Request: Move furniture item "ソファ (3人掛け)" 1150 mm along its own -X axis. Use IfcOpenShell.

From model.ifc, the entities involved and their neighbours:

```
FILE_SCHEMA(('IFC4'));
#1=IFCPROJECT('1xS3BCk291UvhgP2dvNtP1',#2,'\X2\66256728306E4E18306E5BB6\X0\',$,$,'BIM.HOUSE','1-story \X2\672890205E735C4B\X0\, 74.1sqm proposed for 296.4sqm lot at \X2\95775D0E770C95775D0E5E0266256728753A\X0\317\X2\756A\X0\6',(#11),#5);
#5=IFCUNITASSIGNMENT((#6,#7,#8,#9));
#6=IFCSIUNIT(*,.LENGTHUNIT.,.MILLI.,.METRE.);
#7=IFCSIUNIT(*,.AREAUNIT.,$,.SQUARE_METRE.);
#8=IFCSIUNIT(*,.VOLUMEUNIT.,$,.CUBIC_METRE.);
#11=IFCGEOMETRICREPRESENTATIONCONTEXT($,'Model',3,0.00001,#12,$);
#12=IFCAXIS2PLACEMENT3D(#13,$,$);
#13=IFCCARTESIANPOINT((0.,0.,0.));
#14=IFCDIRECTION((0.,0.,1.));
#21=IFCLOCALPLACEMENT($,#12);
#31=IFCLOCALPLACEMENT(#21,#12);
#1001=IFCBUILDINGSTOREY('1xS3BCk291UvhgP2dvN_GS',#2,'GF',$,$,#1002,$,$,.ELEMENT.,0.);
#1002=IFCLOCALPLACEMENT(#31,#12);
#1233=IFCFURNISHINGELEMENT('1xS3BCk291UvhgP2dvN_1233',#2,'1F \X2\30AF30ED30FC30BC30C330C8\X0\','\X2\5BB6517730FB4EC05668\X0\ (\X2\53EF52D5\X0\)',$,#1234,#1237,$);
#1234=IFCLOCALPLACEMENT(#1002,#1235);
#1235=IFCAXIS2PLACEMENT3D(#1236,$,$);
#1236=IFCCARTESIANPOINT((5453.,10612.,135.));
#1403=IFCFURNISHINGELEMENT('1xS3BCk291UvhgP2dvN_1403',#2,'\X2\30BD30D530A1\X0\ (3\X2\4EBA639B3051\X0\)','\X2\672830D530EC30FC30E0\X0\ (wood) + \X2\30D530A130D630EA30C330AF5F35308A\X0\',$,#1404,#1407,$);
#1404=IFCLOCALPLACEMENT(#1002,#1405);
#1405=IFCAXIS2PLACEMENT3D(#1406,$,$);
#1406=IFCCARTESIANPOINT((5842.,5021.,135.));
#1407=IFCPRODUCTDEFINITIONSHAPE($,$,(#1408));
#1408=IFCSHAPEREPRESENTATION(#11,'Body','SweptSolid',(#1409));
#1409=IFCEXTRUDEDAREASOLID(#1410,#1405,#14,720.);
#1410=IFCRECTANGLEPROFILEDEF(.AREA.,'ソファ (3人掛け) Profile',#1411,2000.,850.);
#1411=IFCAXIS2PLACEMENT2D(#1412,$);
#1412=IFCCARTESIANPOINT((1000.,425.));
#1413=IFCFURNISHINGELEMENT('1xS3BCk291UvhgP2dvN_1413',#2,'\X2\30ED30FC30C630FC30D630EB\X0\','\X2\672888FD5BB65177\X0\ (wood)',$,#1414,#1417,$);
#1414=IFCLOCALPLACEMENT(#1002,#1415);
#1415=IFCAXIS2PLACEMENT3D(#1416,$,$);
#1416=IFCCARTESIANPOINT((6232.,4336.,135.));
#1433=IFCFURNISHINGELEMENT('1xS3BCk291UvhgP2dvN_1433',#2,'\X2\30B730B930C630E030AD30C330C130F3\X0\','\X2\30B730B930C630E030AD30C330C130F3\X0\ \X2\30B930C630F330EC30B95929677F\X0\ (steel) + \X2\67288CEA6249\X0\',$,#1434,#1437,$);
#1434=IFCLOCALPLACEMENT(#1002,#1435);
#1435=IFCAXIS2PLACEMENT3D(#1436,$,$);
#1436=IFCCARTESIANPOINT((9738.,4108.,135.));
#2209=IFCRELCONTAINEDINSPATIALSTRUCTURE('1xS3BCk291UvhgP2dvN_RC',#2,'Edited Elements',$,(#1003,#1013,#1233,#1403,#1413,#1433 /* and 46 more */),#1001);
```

```python
import ifcopenshell
import ifcopenshell.api.geometry
import ifcopenshell.util.placement
import ifcopenshell.util.unit

model = ifcopenshell.open("model.ifc")
unit_scale = ifcopenshell.util.unit.calculate_unit_scale(model)

item = model.by_id(1403)
matrix = ifcopenshell.util.placement.get_local_placement(item.ObjectPlacement)
matrix[:3, 3] -= matrix[:3, 0] * 1.15 / unit_scale
ifcopenshell.api.geometry.edit_object_placement(model, product=item, matrix=matrix, is_si=False)

print(ifcopenshell.util.placement.get_local_placement(item.ObjectPlacement).round(3) + 0.0)

model.write("model-out.ifc")
```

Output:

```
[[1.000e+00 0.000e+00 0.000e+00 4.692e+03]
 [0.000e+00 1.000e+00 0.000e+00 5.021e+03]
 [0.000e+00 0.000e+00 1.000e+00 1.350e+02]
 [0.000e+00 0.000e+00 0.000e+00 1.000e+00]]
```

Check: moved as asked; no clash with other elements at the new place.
